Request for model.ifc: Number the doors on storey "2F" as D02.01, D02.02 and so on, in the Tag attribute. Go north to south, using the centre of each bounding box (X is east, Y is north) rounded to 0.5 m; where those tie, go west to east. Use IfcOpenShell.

First a look at what the model holds.

```python
import ifcopenshell
import ifcopenshell.util.element
import ifcopenshell.util.placement

model = ifcopenshell.open("model.ifc")
print(model.schema)
storey = next(s for s in model.by_type("IfcBuildingStorey") if s.Name == "2F")
doors = [e for e in ifcopenshell.util.element.get_decomposition(storey) if e.is_a("IfcDoor")]
for e in sorted(doors, key=lambda e: e.id()):
    origin = ifcopenshell.util.placement.get_local_placement(e.ObjectPlacement)[:3, 3]
    print(e.id(), e.Tag, e.Name, origin.round(2) + 0.0, sep=" | ")
```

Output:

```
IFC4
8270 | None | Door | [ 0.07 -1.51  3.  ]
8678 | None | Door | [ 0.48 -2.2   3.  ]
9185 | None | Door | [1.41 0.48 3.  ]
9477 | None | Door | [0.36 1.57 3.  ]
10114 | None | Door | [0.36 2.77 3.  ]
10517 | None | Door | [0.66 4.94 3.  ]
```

```python
import ifcopenshell
import ifcopenshell.geom
import ifcopenshell.util.element
import ifcopenshell.util.shape

model = ifcopenshell.open("model.ifc")
settings = ifcopenshell.geom.settings()
settings.set("use-world-coords", True)


def centre(element):
    shape = ifcopenshell.geom.create_shape(settings, element)
    return ifcopenshell.util.shape.get_bbox_centroid(shape.geometry)


storey = next(s for s in model.by_type("IfcBuildingStorey") if s.Name == "2F")
doors = [e for e in ifcopenshell.util.element.get_decomposition(storey) if e.is_a("IfcDoor")]

# Insertion points can sit at a corner or the storey origin, so sort by the geometry (in metres).
centres = {e: centre(e) for e in doors}
doors.sort(key=lambda e: (-round(centres[e][1] / 0.5), centres[e][0]))

for i, e in enumerate(doors, start=1):
    number = f"D02.{i:02d}"
    e.Tag = number
    print(e.id(), number)

model.write("model_rev.ifc")
```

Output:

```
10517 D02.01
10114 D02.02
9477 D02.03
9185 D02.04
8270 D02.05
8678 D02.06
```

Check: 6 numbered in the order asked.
